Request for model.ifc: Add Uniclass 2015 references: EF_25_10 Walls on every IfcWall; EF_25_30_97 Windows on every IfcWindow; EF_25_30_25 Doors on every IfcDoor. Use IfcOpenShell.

First a look at what the model holds.

```python
import ifcopenshell

model = ifcopenshell.open("model.ifc")
print(model.schema)
print("classifications:", [c.Name for c in model.by_type("IfcClassification")])
for ifc_class in ("IfcDoor", "IfcRoof", "IfcStair", "IfcWall", "IfcWindow"):
    print(ifc_class, len(model.by_type(ifc_class)))
```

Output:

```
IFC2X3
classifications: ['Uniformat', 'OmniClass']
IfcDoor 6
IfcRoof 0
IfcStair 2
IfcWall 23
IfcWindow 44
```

```python
import ifcopenshell
import ifcopenshell.api.classification

model = ifcopenshell.open("model.ifc")

# IFC2X3 requires Source and Edition and has no link from the project to the system.
system = model.create_entity("IfcClassification", Source="NBS", Edition="2015", Name="Uniclass 2015")

codes = {
    "IfcWall": ("EF_25_10", "Walls"),
    "IfcWindow": ("EF_25_30_97", "Windows"),
    "IfcDoor": ("EF_25_30_25", "Doors"),
}
for ifc_class, (code, name) in codes.items():
    products = model.by_type(ifc_class)
    ifcopenshell.api.classification.add_reference(
        model, products=products, classification=system, identification=code, name=name
    )
    print(code, len(products))

model.write("model_updated.ifc")
```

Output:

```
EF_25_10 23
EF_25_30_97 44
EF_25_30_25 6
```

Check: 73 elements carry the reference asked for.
